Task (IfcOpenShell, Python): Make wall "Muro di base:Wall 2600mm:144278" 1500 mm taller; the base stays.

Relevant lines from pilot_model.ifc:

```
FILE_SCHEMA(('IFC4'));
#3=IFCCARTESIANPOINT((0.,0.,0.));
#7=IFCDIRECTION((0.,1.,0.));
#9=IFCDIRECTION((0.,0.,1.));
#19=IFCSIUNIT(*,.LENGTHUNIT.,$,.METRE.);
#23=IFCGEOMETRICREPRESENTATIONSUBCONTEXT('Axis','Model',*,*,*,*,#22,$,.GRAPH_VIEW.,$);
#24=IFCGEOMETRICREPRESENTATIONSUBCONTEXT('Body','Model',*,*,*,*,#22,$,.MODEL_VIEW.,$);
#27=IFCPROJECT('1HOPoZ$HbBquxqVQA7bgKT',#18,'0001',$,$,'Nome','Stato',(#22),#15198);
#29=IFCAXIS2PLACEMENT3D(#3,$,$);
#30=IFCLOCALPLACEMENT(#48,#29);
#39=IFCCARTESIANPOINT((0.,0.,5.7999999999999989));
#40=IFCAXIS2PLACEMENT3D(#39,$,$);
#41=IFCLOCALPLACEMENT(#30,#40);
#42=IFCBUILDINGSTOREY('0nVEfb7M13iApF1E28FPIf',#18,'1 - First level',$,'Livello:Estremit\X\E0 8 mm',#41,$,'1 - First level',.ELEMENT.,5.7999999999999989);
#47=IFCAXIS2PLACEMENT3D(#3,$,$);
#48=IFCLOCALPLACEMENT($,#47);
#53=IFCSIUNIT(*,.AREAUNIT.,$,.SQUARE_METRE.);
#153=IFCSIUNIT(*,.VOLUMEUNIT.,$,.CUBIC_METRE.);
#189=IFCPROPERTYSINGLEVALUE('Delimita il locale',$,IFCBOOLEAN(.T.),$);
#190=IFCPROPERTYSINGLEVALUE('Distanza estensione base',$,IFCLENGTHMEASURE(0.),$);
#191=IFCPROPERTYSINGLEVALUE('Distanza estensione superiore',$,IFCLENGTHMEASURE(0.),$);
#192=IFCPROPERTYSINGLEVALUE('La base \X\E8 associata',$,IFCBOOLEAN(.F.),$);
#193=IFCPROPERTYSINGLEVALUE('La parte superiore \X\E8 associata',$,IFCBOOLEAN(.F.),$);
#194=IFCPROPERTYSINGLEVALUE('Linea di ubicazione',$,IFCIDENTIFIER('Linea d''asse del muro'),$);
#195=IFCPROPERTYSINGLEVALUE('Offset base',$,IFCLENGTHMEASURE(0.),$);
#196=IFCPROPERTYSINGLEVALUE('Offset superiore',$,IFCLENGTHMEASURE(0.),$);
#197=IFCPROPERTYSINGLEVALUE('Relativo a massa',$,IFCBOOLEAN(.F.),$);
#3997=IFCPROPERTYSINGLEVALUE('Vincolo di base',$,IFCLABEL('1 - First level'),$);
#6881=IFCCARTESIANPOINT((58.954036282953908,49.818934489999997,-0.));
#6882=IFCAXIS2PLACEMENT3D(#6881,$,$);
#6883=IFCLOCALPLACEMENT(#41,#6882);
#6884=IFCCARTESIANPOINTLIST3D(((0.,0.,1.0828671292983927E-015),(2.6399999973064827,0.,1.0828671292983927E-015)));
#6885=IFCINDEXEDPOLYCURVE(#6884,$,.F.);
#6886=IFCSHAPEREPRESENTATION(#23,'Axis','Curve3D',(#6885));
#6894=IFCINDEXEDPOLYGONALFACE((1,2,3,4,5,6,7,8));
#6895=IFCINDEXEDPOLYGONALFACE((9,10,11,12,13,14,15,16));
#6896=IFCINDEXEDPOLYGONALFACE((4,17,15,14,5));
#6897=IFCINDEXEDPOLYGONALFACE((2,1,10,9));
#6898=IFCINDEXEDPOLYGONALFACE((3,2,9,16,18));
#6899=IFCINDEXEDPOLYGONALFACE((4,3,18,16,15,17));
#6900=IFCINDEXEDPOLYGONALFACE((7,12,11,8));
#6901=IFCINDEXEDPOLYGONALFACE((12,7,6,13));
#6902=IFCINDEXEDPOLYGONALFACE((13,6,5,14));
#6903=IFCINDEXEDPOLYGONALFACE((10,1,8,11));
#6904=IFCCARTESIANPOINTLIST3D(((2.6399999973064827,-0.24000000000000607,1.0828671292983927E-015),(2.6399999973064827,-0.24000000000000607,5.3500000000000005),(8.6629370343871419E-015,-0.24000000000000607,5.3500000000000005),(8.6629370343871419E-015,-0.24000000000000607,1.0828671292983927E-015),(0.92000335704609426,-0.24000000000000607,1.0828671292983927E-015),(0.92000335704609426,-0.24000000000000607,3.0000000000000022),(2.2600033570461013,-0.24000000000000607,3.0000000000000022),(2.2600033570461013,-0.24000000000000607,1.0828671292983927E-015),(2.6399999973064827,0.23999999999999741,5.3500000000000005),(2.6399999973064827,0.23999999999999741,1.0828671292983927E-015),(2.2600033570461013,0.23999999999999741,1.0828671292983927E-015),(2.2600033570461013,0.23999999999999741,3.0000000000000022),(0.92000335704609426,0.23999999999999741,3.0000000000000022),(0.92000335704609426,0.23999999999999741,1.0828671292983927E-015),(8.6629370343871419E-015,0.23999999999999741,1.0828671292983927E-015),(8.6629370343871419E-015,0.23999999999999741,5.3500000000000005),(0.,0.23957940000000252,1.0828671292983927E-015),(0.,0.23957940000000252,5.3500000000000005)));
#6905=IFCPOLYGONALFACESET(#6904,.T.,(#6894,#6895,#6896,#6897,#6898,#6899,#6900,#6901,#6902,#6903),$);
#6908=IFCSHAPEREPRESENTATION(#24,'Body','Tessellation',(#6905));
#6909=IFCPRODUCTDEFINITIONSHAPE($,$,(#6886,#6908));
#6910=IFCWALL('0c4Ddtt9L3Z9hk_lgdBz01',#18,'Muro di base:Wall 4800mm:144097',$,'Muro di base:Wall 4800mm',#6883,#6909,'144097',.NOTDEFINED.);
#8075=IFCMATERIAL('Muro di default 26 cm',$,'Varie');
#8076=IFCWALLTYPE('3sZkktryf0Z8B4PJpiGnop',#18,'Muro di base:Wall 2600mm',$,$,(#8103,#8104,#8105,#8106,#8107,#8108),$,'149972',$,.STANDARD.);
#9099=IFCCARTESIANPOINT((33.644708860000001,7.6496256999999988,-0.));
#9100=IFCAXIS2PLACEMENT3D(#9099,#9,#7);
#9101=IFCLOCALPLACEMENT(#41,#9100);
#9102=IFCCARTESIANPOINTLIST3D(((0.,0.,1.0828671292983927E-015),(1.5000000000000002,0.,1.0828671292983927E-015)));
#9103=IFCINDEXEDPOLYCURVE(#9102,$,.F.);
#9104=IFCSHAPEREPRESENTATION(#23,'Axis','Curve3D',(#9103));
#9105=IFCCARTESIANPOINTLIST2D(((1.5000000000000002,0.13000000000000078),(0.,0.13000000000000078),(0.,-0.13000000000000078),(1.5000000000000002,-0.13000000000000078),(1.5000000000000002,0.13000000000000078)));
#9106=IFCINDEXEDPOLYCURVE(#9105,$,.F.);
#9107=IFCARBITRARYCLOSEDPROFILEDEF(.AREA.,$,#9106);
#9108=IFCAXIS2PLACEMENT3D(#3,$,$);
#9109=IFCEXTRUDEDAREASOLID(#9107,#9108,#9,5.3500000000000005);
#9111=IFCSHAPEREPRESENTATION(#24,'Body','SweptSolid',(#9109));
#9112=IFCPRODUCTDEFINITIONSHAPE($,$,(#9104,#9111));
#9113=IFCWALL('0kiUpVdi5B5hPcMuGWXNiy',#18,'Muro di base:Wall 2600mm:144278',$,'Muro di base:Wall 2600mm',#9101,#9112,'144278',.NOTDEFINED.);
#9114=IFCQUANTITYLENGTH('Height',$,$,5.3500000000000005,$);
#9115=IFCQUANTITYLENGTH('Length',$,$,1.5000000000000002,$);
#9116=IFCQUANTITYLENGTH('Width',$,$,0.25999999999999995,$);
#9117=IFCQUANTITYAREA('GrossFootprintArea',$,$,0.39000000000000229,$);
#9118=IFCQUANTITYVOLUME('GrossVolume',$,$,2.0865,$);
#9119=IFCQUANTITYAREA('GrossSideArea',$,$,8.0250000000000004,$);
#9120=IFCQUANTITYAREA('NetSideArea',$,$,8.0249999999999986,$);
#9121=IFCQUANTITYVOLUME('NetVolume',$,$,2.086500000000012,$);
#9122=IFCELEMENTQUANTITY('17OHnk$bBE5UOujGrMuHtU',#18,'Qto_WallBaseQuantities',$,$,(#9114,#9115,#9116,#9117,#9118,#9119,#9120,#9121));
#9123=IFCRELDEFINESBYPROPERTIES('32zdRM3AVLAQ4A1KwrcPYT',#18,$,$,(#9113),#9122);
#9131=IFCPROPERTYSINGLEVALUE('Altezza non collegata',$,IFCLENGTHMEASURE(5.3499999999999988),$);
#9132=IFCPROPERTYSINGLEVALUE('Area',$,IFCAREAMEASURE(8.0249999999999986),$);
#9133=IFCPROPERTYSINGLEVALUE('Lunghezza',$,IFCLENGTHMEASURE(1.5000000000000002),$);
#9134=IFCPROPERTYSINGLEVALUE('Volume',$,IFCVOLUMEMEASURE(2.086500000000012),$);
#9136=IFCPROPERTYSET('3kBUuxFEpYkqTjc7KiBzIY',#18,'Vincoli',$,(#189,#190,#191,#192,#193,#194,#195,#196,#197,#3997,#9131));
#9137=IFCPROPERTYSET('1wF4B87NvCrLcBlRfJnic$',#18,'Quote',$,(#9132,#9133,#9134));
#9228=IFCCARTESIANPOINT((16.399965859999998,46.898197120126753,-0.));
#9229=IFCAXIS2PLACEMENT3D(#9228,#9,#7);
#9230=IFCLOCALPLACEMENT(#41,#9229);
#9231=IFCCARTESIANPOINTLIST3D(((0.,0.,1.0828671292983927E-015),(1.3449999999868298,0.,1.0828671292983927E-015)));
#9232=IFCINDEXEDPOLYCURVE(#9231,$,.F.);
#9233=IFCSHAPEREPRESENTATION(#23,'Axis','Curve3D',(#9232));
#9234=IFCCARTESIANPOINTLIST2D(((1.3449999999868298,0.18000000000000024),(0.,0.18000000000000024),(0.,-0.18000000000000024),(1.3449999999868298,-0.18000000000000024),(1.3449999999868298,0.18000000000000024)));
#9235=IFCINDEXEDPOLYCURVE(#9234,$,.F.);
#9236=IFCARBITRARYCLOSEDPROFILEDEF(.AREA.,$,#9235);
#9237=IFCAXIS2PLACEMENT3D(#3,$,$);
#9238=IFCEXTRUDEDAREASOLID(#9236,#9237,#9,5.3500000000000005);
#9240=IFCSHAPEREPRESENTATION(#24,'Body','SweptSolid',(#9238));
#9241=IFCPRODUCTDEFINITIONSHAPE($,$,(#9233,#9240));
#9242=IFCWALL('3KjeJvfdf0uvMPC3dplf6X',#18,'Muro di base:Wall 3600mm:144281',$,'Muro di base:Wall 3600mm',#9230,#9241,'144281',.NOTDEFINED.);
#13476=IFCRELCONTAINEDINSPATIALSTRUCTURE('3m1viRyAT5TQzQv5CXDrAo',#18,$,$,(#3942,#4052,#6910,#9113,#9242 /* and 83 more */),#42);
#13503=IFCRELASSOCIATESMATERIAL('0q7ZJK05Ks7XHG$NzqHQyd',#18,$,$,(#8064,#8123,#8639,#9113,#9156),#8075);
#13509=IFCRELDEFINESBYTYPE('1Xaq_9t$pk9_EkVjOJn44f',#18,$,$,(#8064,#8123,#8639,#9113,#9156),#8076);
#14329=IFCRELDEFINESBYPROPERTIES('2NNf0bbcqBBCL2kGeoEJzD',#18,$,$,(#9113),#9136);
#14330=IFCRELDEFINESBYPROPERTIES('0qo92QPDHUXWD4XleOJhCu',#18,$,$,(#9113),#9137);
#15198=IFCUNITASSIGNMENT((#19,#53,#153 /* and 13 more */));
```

```python
import ifcopenshell
import ifcopenshell.api.pset
import ifcopenshell.geom
import ifcopenshell.util.element
import ifcopenshell.util.representation
import ifcopenshell.util.shape
import ifcopenshell.util.unit

model = ifcopenshell.open("pilot_model.ifc")
unit_scale = ifcopenshell.util.unit.calculate_unit_scale(model)
area_scale = ifcopenshell.util.unit.calculate_unit_scale(model, "AREAUNIT")
volume_scale = ifcopenshell.util.unit.calculate_unit_scale(model, "VOLUMEUNIT")
settings = ifcopenshell.geom.settings()


def volume(element):
    """Net volume in cubic metres, openings subtracted."""
    shape = ifcopenshell.geom.create_shape(settings, element)
    return ifcopenshell.util.shape.get_volume(shape.geometry)


wall = model.by_guid("0kiUpVdi5B5hPcMuGWXNiy")
before = volume(wall)

body = ifcopenshell.util.representation.get_representation(wall, "Model", "Body")
solid = body.Items[0]
old_height = solid.Depth
solid.Depth += 1.5 / unit_scale
after = volume(wall)
thickness = 0.26  # wall thickness in metres

# Update the stored height, areas and volumes.
qto = model.by_id(ifcopenshell.util.element.get_pset(wall, "Qto_WallBaseQuantities", should_inherit=False)["id"])
ifcopenshell.api.pset.edit_qto(model, qto=qto, properties={
    "Height": solid.Depth,
    "GrossVolume": ifcopenshell.util.element.get_pset(wall, "Qto_WallBaseQuantities", "GrossVolume") * solid.Depth / old_height,
    "GrossSideArea": ifcopenshell.util.element.get_pset(wall, "Qto_WallBaseQuantities", "GrossSideArea") * solid.Depth / old_height,
    "NetSideArea": after / thickness / area_scale,
    "NetVolume": after / volume_scale,
})
pset = model.by_id(ifcopenshell.util.element.get_pset(wall, "Vincoli", should_inherit=False)["id"])
ifcopenshell.api.pset.edit_pset(model, pset=pset, properties={
    "Altezza non collegata": model.create_entity("IfcLengthMeasure", solid.Depth),
})
pset = model.by_id(ifcopenshell.util.element.get_pset(wall, "Quote", should_inherit=False)["id"])
ifcopenshell.api.pset.edit_pset(model, pset=pset, properties={
    "Area": model.create_entity("IfcAreaMeasure", after / thickness / area_scale),
    "Volume": model.create_entity("IfcVolumeMeasure", after / volume_scale),
})

print(f"height {old_height:g} -> {solid.Depth:g}, volume {before:.3f} -> {after:.3f} m3")

model.write("pilot_model_updated.ifc")
```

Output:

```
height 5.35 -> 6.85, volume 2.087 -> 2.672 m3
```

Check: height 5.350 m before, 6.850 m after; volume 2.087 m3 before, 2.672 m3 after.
